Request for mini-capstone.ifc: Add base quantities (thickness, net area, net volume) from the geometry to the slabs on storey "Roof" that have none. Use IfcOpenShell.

First a look at what the model holds.

```python
import ifcopenshell
import ifcopenshell.util.element
import ifcopenshell.util.unit

model = ifcopenshell.open("mini-capstone.ifc")
print(model.schema)
for unit_type in ("LENGTHUNIT", "AREAUNIT", "VOLUMEUNIT"):
    print(unit_type, ifcopenshell.util.unit.calculate_unit_scale(model, unit_type))
storey = next(s for s in model.by_type("IfcBuildingStorey") if s.Name == "Roof")
slabs = [e for e in ifcopenshell.util.element.get_decomposition(storey) if e.is_a("IfcSlab")]
for e in sorted(slabs, key=lambda e: e.id()):
    print(e.id(), e.is_a(), e.Name, list(ifcopenshell.util.element.get_psets(e, qtos_only=True)), sep=" | ")
```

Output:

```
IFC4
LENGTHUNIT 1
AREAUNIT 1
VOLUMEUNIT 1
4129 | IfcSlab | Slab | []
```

```python
import ifcopenshell
import ifcopenshell.api.pset
import ifcopenshell.geom
import ifcopenshell.util.element
import ifcopenshell.util.shape
import ifcopenshell.util.unit

model = ifcopenshell.open("mini-capstone.ifc")
unit_scale = ifcopenshell.util.unit.calculate_unit_scale(model)
area_scale = ifcopenshell.util.unit.calculate_unit_scale(model, "AREAUNIT")
volume_scale = ifcopenshell.util.unit.calculate_unit_scale(model, "VOLUMEUNIT")
settings = ifcopenshell.geom.settings()

storey = next(s for s in model.by_type("IfcBuildingStorey") if s.Name == "Roof")
slabs = [e for e in ifcopenshell.util.element.get_decomposition(storey) if e.is_a("IfcSlab")]

for e in sorted(slabs, key=lambda e: e.id()):
    if ifcopenshell.util.element.get_psets(e, qtos_only=True, should_inherit=False):
        continue
    # Geometry comes back in metres, in the element's own axes.
    shape = ifcopenshell.geom.create_shape(settings, e)
    values = {
        "Width": ifcopenshell.util.shape.get_z(shape.geometry) / unit_scale,
        "NetArea": ifcopenshell.util.shape.get_footprint_area(shape.geometry) / area_scale,
        "NetVolume": ifcopenshell.util.shape.get_volume(shape.geometry) / volume_scale,
    }
    qto = ifcopenshell.api.pset.add_qto(model, product=e, name="Qto_SlabBaseQuantities")
    ifcopenshell.api.pset.edit_qto(model, qto=qto, properties=values)
    print(e.id(), {k: round(v, 3) for k, v in values.items()})

model.write("mini-capstone_updated.ifc")
```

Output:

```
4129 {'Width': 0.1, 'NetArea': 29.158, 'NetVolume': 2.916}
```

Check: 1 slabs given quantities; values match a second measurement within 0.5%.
